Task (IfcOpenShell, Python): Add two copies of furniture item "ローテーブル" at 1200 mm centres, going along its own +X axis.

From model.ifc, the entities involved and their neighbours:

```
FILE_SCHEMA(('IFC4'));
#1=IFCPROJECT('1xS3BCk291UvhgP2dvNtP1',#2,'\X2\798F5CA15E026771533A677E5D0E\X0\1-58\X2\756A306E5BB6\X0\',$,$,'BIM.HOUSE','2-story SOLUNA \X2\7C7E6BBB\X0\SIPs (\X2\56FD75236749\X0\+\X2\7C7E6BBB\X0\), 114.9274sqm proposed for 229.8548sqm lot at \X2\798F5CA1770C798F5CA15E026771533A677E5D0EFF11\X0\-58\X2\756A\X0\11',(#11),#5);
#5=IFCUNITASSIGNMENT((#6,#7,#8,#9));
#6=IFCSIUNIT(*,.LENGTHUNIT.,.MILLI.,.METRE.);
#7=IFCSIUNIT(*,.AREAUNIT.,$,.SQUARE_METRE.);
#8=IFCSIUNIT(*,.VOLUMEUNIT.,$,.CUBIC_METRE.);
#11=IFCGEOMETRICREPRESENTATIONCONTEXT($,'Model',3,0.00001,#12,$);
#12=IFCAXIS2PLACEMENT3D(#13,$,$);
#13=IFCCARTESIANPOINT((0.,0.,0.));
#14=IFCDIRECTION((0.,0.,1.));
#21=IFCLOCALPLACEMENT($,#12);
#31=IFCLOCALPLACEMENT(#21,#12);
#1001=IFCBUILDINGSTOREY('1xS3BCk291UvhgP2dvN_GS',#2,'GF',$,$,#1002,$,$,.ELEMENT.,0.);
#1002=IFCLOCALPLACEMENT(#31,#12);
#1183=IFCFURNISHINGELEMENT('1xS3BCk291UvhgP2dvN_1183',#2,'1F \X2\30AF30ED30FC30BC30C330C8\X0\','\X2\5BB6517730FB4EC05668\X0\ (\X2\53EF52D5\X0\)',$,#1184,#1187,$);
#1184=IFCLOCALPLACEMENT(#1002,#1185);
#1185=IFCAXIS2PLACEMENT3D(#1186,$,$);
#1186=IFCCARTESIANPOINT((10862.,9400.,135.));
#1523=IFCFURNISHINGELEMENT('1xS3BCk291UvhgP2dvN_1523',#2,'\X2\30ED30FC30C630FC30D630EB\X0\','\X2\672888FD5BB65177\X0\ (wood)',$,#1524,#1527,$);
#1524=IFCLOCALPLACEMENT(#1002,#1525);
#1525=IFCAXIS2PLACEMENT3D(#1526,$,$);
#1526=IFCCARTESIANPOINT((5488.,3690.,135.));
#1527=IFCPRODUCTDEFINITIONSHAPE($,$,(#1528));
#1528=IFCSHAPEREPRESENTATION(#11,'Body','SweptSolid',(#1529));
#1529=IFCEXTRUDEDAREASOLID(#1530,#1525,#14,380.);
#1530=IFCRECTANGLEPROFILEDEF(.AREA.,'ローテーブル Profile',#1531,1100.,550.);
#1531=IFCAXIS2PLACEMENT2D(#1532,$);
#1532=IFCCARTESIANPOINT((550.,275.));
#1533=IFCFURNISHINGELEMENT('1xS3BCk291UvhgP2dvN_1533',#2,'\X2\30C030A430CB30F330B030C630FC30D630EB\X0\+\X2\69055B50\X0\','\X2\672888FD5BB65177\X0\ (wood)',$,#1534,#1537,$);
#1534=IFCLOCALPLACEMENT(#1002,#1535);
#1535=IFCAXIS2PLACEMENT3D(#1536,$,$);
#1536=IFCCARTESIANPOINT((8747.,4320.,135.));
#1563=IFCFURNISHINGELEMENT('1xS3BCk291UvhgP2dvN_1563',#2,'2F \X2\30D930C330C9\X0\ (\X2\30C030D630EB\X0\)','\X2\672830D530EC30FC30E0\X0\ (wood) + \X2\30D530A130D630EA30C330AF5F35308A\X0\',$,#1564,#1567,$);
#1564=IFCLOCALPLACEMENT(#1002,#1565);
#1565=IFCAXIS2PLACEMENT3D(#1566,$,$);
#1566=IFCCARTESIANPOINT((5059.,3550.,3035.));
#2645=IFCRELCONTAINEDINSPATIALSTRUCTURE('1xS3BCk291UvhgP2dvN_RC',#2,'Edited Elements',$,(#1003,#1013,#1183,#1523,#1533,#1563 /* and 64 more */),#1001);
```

```python
import ifcopenshell
import ifcopenshell.api.geometry
import ifcopenshell.api.root
import ifcopenshell.util.element
import ifcopenshell.util.placement
import ifcopenshell.util.unit

model = ifcopenshell.open("model.ifc")
unit_scale = ifcopenshell.util.unit.calculate_unit_scale(model)


def reuse_history(source, copy):
    """copy_class also copies each property set's owner history, people and application; keep the originals."""
    for rel in copy.IsDefinedBy:
        if rel.is_a("IfcRelDefinesByProperties") and (history := rel.RelatingPropertyDefinition.OwnerHistory):
            rel.RelatingPropertyDefinition.OwnerHistory = source.OwnerHistory
            ifcopenshell.util.element.remove_deep2(model, history)


source = model.by_guid("1xS3BCk291UvhgP2dvN_1523")
base = ifcopenshell.util.placement.get_local_placement(source.ObjectPlacement)
step = base[:3, 0] * 1.2 / unit_scale

for i in range(1, 3):
    copy = ifcopenshell.api.root.copy_class(model, product=source)
    copy.Representation = ifcopenshell.util.element.copy_deep(
        model, source.Representation, exclude=["IfcGeometricRepresentationContext", "IfcRepresentationMap"]
    )
    reuse_history(source, copy)
    matrix = base.copy()
    matrix[:3, 3] += i * step
    print("added at", matrix[:3, 3].round(3) + 0.0)
    ifcopenshell.api.geometry.edit_object_placement(model, product=copy, matrix=matrix, is_si=False)

model.write("model_v2.ifc")
```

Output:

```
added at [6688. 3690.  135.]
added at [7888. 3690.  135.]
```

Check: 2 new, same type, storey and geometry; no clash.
